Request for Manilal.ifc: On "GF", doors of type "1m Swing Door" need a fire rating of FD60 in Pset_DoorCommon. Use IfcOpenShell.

First a look at what the model holds.

```python
import ifcopenshell
import ifcopenshell.util.element

model = ifcopenshell.open("Manilal.ifc")
print(model.schema)
storey = next(s for s in model.by_type("IfcBuildingStorey") if s.Name == "GF")
doors = [e for e in ifcopenshell.util.element.get_decomposition(storey) if e.is_a("IfcDoor")]
seen = {}
for e in doors:
    element_type = ifcopenshell.util.element.get_type(e)
    key = (element_type.Name if element_type != e and element_type else None, ifcopenshell.util.element.get_pset(e, "Pset_DoorCommon", "FireRating"))
    seen[key] = seen.get(key, 0) + 1
for (name, value), count in sorted(seen.items(), key=str):
    print(count, "x", name, "|", value)
```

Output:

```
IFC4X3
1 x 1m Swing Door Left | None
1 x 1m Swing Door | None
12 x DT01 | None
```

```python
import ifcopenshell
import ifcopenshell.api.pset
import ifcopenshell.util.element

model = ifcopenshell.open("Manilal.ifc")

storey = next(s for s in model.by_type("IfcBuildingStorey") if s.Name == "GF")
doors = [e for e in ifcopenshell.util.element.get_decomposition(storey) if e.is_a("IfcDoor")]

count = 0
for e in doors:
    element_type = ifcopenshell.util.element.get_type(e)
    if element_type in (None, e) or element_type.Name != "1m Swing Door":
        continue
    # add_pset returns the element's existing set when there is one.
    pset = ifcopenshell.api.pset.add_pset(model, product=e, name="Pset_DoorCommon")
    ifcopenshell.api.pset.edit_pset(model, pset=pset, properties={"FireRating": "FD60"})
    count += 1

print(count, "doors updated")

model.write("Manilal_updated.ifc")
```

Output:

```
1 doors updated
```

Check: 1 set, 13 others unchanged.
